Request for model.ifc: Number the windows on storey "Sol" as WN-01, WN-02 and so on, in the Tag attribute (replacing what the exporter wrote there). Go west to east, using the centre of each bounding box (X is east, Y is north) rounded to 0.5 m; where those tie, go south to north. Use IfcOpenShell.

First a look at what the model holds.

```python
import ifcopenshell
import ifcopenshell.util.element
import ifcopenshell.util.placement

model = ifcopenshell.open("model.ifc")
print(model.schema)
storey = next(s for s in model.by_type("IfcBuildingStorey") if s.Name == "Sol")
windows = [e for e in ifcopenshell.util.element.get_decomposition(storey) if e.is_a("IfcWindow")]
for e in sorted(windows, key=lambda e: e.id()):
    origin = ifcopenshell.util.placement.get_local_placement(e.ObjectPlacement)[:3, 3]
    print(e.id(), e.Tag, e.Name, origin.round(2) + 0.0, sep=" | ")
```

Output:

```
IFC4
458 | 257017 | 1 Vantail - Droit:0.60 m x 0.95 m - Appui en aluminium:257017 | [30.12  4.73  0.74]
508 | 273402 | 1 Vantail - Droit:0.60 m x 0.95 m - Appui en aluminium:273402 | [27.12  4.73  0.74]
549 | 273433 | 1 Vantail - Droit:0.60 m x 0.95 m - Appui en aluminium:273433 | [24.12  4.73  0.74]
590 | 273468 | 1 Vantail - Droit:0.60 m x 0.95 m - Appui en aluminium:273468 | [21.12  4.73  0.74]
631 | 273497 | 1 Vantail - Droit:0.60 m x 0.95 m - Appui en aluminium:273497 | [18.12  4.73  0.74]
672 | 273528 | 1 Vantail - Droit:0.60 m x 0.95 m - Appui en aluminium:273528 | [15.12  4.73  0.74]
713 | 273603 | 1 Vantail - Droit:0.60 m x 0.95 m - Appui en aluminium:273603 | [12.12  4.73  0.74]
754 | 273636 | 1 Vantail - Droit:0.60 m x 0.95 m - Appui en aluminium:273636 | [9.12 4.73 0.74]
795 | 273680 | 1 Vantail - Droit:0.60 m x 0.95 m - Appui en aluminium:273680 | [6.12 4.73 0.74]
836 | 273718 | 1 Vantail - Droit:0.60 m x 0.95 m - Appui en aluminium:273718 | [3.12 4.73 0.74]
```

```python
import ifcopenshell
import ifcopenshell.geom
import ifcopenshell.util.element
import ifcopenshell.util.shape

model = ifcopenshell.open("model.ifc")
settings = ifcopenshell.geom.settings()
settings.set("use-world-coords", True)


def centre(element):
    shape = ifcopenshell.geom.create_shape(settings, element)
    return ifcopenshell.util.shape.get_bbox_centroid(shape.geometry)


storey = next(s for s in model.by_type("IfcBuildingStorey") if s.Name == "Sol")
windows = [e for e in ifcopenshell.util.element.get_decomposition(storey) if e.is_a("IfcWindow")]

# Insertion points can sit at a corner or the storey origin, so sort by the geometry (in metres).
centres = {e: centre(e) for e in windows}
windows.sort(key=lambda e: (round(centres[e][0] / 0.5), centres[e][1]))

for i, e in enumerate(windows, start=1):
    number = f"WN-{i:02d}"
    e.Tag = number
    print(e.id(), number)

model.write("model_v2.ifc")
```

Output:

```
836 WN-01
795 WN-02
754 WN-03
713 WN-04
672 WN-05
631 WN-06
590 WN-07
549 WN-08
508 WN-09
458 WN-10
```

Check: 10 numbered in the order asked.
